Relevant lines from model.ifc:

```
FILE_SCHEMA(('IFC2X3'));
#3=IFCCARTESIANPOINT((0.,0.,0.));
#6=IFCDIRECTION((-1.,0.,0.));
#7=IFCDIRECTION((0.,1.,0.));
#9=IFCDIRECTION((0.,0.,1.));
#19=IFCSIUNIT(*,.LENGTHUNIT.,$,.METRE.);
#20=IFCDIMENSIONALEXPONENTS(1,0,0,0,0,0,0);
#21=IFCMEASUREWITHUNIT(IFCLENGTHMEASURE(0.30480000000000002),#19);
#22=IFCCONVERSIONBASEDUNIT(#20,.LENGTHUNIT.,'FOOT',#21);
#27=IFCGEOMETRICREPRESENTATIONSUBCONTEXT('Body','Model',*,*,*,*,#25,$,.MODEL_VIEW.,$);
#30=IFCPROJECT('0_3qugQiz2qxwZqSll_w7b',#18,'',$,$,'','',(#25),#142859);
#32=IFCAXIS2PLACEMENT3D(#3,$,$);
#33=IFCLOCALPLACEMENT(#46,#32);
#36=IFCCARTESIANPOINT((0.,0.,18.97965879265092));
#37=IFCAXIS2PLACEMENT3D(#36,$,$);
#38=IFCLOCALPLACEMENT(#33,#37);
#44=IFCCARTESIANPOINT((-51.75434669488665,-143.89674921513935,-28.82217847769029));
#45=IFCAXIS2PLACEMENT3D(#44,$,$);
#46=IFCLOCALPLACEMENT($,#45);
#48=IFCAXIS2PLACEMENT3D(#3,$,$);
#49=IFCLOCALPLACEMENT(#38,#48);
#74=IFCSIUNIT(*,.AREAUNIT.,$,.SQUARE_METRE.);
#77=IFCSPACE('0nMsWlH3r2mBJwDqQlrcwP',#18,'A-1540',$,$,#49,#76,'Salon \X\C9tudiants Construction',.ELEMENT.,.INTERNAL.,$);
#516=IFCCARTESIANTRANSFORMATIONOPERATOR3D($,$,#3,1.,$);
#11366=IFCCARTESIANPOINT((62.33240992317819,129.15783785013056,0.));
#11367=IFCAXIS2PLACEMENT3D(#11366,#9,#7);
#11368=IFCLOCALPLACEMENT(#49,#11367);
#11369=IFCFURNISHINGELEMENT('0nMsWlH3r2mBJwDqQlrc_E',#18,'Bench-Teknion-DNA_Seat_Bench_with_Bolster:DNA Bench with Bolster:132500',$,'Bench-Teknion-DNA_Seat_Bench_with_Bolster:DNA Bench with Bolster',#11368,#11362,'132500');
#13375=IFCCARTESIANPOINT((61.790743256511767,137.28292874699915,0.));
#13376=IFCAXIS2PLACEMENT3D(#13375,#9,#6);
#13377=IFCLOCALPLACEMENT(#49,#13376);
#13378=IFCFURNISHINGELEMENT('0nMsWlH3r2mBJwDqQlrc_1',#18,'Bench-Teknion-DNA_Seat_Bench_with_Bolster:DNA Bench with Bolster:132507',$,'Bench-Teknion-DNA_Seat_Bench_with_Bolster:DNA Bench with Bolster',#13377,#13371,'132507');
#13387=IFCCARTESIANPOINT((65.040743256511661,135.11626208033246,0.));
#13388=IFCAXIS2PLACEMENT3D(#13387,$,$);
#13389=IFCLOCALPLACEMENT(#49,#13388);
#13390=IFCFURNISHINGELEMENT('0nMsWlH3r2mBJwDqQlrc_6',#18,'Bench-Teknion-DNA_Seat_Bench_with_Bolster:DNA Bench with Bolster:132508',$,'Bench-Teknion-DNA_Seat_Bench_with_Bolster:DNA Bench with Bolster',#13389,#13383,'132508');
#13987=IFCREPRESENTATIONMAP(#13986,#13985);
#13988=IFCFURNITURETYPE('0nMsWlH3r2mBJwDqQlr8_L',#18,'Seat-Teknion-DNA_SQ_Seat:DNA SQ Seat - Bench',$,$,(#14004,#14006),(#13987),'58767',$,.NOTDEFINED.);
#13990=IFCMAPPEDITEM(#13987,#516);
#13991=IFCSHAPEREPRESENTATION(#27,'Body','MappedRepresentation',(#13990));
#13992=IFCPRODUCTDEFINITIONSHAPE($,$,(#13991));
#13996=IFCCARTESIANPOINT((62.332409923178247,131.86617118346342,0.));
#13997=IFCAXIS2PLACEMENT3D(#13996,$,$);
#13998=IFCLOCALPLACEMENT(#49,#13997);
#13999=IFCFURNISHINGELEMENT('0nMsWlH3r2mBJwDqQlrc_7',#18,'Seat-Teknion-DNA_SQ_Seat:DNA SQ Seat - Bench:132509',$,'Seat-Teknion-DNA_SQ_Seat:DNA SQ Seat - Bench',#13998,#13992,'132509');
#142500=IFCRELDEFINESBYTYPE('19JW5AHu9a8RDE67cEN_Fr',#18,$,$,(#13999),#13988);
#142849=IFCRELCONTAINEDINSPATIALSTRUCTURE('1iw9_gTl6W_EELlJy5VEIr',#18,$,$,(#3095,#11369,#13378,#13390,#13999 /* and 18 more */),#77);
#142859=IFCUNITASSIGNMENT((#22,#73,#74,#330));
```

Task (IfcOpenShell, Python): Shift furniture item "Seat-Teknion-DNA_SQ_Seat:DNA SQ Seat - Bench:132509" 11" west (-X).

```python
import ifcopenshell
import ifcopenshell.api.geometry
import ifcopenshell.util.placement
import ifcopenshell.util.unit

model = ifcopenshell.open("model.ifc")
unit_scale = ifcopenshell.util.unit.calculate_unit_scale(model)

item = model.by_guid("0nMsWlH3r2mBJwDqQlrc_7")
matrix = ifcopenshell.util.placement.get_local_placement(item.ObjectPlacement)
matrix[0, 3] -= 11 * 0.0254 / unit_scale
ifcopenshell.api.geometry.edit_object_placement(model, product=item, matrix=matrix, is_si=False)

print(ifcopenshell.util.placement.get_local_placement(item.ObjectPlacement).round(3) + 0.0)

model.write("model-out.ifc")
```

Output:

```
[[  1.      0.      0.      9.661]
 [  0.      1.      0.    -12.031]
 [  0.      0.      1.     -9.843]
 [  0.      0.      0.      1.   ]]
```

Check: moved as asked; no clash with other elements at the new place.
